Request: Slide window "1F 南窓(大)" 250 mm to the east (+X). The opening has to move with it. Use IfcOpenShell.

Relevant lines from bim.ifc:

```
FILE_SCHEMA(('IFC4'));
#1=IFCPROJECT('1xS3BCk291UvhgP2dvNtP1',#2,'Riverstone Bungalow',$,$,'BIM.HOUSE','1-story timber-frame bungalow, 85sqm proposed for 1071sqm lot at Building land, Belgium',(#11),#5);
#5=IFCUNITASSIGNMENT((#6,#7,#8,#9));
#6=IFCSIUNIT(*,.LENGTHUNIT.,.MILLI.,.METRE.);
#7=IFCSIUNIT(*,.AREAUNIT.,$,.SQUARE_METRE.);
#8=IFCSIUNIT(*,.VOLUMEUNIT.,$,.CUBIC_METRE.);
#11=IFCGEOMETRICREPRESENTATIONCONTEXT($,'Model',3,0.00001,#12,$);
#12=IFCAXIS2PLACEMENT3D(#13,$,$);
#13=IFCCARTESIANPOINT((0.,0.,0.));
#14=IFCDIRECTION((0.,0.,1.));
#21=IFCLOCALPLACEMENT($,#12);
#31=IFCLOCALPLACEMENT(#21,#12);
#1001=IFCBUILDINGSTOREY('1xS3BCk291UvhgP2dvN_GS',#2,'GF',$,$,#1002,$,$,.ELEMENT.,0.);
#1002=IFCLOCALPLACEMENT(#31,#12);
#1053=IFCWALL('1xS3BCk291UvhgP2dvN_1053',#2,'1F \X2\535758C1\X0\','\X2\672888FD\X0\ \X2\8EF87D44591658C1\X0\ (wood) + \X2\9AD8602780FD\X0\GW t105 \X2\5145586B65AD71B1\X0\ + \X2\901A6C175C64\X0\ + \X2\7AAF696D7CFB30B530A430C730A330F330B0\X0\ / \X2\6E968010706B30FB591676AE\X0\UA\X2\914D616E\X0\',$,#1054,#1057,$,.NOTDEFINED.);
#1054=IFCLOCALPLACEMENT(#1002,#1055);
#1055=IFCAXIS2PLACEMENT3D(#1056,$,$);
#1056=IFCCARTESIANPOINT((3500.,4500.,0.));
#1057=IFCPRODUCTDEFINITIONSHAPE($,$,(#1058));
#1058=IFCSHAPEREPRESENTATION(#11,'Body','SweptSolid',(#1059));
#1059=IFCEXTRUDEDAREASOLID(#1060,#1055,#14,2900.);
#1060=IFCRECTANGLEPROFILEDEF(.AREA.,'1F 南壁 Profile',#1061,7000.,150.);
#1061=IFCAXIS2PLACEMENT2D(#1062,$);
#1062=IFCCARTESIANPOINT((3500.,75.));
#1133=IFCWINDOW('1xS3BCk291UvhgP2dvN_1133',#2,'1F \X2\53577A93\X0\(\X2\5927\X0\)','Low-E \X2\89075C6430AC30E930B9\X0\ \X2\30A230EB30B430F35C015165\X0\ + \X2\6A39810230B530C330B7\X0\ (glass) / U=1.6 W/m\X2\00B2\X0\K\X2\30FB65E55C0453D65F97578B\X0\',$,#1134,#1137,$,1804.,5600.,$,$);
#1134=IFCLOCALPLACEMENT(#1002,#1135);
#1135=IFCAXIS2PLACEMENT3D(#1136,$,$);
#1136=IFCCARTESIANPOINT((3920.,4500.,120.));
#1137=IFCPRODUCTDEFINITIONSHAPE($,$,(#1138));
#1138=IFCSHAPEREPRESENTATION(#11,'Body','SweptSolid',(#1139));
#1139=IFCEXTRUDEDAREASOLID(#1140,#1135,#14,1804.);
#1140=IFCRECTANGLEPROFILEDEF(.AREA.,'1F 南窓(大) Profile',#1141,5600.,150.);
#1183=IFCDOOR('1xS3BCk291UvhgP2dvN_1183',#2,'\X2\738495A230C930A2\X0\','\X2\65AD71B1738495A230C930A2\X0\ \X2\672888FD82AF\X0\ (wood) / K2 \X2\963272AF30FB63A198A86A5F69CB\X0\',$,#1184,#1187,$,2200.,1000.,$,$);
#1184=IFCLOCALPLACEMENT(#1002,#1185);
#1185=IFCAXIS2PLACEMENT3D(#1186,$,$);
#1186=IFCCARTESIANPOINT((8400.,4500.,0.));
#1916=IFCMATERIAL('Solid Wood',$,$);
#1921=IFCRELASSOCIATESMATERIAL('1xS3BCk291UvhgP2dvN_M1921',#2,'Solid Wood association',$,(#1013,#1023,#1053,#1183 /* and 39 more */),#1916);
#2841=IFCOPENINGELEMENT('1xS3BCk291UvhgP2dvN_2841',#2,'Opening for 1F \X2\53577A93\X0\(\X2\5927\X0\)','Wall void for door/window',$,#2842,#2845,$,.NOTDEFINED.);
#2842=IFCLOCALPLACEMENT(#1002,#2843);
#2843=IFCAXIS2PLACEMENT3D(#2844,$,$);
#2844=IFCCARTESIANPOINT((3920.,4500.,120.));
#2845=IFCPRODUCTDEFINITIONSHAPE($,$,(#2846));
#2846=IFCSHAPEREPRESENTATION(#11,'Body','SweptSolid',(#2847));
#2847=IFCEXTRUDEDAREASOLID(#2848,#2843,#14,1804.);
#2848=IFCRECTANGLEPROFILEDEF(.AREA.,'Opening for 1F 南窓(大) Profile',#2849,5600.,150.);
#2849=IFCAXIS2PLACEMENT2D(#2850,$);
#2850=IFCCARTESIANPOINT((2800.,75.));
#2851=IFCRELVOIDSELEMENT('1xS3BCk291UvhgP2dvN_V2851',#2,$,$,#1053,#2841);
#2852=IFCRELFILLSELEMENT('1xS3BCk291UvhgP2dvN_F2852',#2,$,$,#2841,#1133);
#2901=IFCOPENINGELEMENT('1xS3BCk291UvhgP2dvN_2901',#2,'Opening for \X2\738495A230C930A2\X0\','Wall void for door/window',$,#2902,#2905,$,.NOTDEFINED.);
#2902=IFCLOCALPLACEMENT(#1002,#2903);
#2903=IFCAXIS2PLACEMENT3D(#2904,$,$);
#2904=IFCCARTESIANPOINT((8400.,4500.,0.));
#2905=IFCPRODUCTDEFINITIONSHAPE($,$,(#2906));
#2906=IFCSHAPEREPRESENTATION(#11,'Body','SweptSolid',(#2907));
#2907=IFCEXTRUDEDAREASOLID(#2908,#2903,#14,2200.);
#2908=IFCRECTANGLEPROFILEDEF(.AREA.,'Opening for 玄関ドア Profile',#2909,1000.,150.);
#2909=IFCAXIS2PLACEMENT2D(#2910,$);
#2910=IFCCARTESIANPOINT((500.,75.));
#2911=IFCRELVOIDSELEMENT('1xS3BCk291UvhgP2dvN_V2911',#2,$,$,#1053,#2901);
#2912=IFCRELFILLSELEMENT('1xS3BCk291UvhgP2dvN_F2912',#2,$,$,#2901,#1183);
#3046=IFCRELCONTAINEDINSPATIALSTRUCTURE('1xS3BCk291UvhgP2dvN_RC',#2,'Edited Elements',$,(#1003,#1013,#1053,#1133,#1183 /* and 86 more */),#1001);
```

```python
import ifcopenshell
import ifcopenshell.api.geometry
import ifcopenshell.util.placement

model = ifcopenshell.open("bim.ifc")

window = model.by_id(1133)
opening = window.FillsVoids[0].RelatingOpeningElement
wall = opening.VoidsElements[0].RelatingBuildingElement

wall_matrix = ifcopenshell.util.placement.get_local_placement(wall.ObjectPlacement)
shift = wall_matrix[:3, 0] * 250.0
before = ifcopenshell.util.placement.get_local_placement(window.ObjectPlacement)[:3, 3].copy()

# The window is not placed relative to its opening, so move both.
for product in (opening, window):
    matrix = ifcopenshell.util.placement.get_local_placement(product.ObjectPlacement)
    matrix[:3, 3] += shift
    ifcopenshell.api.geometry.edit_object_placement(model, product=product, matrix=matrix, is_si=False)

after = ifcopenshell.util.placement.get_local_placement(window.ObjectPlacement)[:3, 3]
print("window moved by", (after - before).round(3) + 0.0)

model.write("bim_updated.ifc")
```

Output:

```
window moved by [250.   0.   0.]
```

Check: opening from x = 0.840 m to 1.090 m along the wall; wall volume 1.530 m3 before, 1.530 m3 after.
